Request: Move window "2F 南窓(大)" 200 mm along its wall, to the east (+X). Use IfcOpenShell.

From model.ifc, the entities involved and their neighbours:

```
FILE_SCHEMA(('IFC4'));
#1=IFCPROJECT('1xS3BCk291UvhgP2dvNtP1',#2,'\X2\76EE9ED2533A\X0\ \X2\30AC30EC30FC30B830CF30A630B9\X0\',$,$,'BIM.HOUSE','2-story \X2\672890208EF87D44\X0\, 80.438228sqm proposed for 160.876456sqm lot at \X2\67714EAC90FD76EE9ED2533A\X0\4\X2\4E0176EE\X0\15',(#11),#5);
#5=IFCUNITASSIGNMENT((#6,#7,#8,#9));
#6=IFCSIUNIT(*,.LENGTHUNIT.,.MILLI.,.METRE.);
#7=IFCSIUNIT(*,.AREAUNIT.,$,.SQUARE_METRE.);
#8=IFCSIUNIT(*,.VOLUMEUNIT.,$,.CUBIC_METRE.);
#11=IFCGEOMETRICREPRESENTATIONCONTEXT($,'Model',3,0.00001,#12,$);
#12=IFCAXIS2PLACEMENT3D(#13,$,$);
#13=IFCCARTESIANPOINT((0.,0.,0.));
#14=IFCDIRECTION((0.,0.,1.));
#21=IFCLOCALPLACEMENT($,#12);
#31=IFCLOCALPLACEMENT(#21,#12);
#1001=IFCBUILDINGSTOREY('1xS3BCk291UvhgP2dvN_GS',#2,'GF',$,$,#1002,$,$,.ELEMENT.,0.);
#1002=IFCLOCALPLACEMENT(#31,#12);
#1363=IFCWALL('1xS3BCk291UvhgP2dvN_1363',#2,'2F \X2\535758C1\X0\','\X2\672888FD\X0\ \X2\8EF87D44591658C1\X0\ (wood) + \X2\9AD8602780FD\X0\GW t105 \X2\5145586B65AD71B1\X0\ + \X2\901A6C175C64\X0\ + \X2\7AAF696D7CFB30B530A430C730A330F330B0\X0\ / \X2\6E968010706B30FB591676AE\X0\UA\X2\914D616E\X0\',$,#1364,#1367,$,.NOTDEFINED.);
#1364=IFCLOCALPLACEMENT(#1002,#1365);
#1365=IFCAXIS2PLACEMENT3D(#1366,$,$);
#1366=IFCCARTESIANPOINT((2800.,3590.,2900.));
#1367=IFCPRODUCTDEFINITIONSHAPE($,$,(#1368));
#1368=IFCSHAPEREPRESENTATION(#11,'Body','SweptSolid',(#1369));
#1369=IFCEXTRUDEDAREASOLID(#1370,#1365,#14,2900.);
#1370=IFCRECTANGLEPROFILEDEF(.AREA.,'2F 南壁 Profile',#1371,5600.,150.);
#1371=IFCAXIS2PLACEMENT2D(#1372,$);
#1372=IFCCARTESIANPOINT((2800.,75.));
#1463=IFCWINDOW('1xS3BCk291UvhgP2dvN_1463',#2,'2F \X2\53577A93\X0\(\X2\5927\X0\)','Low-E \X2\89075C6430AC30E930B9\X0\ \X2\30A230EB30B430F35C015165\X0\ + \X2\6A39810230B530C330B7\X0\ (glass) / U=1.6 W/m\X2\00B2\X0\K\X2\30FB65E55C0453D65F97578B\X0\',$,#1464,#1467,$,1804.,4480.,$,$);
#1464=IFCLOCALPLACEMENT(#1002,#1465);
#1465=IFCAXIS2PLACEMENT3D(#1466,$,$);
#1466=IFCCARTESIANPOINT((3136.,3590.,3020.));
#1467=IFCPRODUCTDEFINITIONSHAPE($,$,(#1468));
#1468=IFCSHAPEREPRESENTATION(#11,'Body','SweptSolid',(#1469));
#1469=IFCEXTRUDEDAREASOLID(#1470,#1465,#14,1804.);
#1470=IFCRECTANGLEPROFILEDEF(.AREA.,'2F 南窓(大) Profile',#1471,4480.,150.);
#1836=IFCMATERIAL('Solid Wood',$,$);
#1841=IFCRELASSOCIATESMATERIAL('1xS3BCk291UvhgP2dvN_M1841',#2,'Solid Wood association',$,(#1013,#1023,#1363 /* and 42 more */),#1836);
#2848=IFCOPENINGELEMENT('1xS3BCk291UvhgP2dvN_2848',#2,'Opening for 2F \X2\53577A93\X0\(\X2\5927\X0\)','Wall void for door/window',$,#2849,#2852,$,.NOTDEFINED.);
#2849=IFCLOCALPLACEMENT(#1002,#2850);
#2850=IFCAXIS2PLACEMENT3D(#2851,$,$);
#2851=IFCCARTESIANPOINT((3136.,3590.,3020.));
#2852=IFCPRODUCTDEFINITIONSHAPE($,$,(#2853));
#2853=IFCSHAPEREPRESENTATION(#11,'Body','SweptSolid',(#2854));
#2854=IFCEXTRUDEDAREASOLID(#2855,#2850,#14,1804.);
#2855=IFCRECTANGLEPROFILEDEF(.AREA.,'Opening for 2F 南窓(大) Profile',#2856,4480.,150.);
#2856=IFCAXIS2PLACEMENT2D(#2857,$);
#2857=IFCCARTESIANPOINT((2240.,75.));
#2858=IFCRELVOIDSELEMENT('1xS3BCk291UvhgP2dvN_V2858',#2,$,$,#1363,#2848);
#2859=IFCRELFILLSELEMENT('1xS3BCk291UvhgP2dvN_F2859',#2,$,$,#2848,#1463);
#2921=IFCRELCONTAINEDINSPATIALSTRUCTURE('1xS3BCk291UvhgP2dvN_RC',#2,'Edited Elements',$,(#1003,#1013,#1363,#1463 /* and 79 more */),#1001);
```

```python
import ifcopenshell
import ifcopenshell.api.geometry
import ifcopenshell.util.placement
import ifcopenshell.util.unit

model = ifcopenshell.open("model.ifc")
unit_scale = ifcopenshell.util.unit.calculate_unit_scale(model)

window = model.by_guid("1xS3BCk291UvhgP2dvN_1463")
opening = window.FillsVoids[0].RelatingOpeningElement
wall = opening.VoidsElements[0].RelatingBuildingElement

wall_matrix = ifcopenshell.util.placement.get_local_placement(wall.ObjectPlacement)
shift = wall_matrix[:3, 0] * 0.2 / unit_scale
before = ifcopenshell.util.placement.get_local_placement(window.ObjectPlacement)[:3, 3].copy()

# The window is not placed relative to its opening, so move both.
for product in (opening, window):
    matrix = ifcopenshell.util.placement.get_local_placement(product.ObjectPlacement)
    matrix[:3, 3] += shift
    ifcopenshell.api.geometry.edit_object_placement(model, product=product, matrix=matrix, is_si=False)

after = ifcopenshell.util.placement.get_local_placement(window.ObjectPlacement)[:3, 3]
print("window moved by", (after - before).round(3) + 0.0)

model.write("model_v2.ifc")
```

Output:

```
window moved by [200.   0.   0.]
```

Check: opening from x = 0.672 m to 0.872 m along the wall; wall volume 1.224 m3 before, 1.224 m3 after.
